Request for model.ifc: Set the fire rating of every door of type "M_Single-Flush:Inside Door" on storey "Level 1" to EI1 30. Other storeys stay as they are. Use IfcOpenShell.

First a look at what the model holds.

```python
import ifcopenshell
import ifcopenshell.util.element

model = ifcopenshell.open("model.ifc")
print(model.schema)
storey = next(s for s in model.by_type("IfcBuildingStorey") if s.Name == "Level 1")
doors = [e for e in ifcopenshell.util.element.get_decomposition(storey) if e.is_a("IfcDoor")]
seen = {}
for e in doors:
    element_type = ifcopenshell.util.element.get_type(e)
    key = (element_type.Name if element_type != e and element_type else None, ifcopenshell.util.element.get_pset(e, "Pset_DoorCommon", "FireRating"))
    seen[key] = seen.get(key, 0) + 1
for (name, value), count in sorted(seen.items(), key=str):
    print(count, "x", name, "|", value)
```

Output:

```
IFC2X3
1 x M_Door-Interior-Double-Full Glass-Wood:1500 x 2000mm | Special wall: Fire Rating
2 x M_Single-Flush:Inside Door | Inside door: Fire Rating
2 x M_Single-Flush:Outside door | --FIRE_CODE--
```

```python
import ifcopenshell
import ifcopenshell.api.pset
import ifcopenshell.util.element

model = ifcopenshell.open("model.ifc")

storey = next(s for s in model.by_type("IfcBuildingStorey") if s.Name == "Level 1")
doors = [e for e in ifcopenshell.util.element.get_decomposition(storey) if e.is_a("IfcDoor")]

count = 0
for e in doors:
    element_type = ifcopenshell.util.element.get_type(e)
    if element_type in (None, e) or element_type.Name != "M_Single-Flush:Inside Door":
        continue
    # add_pset returns the element's existing set when there is one.
    pset = ifcopenshell.api.pset.add_pset(model, product=e, name="Pset_DoorCommon")
    ifcopenshell.api.pset.edit_pset(model, pset=pset, properties={"FireRating": "EI1 30"})
    count += 1

print(count, "doors updated")

model.write("model_v2.ifc")
```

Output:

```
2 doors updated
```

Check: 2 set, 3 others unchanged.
